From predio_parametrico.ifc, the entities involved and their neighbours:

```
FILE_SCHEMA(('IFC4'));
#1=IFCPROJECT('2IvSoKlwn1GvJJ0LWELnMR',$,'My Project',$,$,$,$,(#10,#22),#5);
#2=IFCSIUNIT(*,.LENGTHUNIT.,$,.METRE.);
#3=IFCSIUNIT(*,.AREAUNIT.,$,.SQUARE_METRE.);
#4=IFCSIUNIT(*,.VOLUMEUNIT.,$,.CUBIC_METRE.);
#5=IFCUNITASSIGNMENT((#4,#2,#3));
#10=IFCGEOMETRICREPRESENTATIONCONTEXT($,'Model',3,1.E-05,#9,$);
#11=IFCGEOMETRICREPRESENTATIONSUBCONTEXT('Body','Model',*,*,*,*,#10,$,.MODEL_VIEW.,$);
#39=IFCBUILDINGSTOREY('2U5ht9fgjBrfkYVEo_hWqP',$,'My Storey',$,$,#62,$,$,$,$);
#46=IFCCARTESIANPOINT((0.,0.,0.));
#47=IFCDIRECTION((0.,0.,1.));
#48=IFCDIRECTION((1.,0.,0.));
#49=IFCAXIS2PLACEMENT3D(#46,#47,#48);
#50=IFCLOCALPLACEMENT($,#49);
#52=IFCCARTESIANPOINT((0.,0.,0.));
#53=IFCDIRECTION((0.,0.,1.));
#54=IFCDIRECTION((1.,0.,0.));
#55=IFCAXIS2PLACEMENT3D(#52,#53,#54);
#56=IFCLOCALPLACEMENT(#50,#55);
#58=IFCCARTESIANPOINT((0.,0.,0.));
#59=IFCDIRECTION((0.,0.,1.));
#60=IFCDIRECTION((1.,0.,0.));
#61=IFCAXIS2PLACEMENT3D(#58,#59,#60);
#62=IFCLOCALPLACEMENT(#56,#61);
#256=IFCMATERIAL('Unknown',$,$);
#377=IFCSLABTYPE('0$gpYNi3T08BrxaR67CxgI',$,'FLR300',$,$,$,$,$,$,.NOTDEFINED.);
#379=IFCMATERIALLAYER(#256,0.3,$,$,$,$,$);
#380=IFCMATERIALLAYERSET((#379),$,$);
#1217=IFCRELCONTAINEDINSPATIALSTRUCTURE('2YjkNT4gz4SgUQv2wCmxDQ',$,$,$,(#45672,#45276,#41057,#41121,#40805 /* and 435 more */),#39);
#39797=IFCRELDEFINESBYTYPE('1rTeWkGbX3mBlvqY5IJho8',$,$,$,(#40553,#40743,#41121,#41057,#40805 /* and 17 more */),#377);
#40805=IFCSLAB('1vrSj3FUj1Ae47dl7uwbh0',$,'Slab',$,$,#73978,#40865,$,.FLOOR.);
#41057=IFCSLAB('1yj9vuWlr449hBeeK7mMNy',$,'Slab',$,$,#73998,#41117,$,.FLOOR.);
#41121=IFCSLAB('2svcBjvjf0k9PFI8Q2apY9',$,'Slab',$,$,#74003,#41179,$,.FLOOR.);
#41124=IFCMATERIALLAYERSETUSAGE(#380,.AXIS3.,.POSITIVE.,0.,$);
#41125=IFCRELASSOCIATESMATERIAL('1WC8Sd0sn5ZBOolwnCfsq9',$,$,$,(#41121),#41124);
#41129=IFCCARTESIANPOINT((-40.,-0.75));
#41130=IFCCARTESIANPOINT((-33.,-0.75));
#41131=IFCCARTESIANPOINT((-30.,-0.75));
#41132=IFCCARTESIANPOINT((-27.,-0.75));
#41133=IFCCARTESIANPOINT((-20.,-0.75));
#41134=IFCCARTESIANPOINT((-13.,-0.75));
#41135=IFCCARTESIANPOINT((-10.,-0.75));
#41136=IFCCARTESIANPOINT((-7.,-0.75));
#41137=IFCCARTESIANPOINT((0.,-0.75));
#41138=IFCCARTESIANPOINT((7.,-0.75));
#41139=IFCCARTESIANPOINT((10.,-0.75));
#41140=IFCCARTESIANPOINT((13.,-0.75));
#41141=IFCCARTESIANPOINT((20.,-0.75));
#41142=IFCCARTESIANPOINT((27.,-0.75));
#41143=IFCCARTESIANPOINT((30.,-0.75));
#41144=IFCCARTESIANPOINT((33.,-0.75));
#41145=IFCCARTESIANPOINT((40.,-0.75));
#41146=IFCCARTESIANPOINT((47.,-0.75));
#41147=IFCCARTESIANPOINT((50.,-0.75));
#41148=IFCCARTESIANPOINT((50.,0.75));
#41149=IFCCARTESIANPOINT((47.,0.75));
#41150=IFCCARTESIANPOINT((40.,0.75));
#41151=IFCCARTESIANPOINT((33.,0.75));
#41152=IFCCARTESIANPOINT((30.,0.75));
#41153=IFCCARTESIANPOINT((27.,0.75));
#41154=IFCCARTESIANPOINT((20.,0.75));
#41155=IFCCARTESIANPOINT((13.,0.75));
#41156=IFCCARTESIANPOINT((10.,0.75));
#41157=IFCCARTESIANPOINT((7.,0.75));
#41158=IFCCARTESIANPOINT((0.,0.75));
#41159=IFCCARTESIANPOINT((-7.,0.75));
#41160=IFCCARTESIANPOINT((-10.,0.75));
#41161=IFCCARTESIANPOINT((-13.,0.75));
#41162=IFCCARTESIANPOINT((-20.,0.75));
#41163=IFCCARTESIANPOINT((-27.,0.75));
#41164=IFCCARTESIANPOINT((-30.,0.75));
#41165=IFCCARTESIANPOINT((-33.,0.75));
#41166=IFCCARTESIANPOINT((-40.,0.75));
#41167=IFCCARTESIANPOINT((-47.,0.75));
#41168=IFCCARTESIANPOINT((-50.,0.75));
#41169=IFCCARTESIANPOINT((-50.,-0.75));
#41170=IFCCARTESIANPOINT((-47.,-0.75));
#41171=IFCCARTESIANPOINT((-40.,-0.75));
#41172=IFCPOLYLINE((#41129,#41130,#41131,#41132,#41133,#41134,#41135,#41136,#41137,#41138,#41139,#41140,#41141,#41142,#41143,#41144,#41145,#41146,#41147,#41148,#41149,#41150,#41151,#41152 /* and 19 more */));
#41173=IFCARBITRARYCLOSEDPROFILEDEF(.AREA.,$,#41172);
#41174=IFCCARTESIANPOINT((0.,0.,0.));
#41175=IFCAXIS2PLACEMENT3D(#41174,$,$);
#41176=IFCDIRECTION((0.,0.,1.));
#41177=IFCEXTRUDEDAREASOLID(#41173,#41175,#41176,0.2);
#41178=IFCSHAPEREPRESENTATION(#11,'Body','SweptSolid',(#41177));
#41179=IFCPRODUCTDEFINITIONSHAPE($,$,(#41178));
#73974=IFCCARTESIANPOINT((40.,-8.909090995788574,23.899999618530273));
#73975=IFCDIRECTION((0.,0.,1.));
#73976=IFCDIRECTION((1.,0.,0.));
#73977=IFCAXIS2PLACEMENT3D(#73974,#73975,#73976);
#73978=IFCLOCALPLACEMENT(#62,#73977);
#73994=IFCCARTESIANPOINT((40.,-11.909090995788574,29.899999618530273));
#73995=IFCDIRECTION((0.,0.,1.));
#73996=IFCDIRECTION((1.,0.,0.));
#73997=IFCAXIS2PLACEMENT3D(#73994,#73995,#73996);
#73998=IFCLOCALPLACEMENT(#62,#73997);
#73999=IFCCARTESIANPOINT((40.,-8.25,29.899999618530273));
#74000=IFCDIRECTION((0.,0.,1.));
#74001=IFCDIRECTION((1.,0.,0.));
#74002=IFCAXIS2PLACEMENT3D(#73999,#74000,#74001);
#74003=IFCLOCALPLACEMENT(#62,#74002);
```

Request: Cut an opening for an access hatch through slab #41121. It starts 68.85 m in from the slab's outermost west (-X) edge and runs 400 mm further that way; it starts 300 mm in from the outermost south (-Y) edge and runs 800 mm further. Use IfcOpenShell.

```python
import numpy as np
import ifcopenshell
import ifcopenshell.api.feature
import ifcopenshell.api.geometry
import ifcopenshell.api.root
import ifcopenshell.geom
import ifcopenshell.util.placement
import ifcopenshell.util.representation
import ifcopenshell.util.shape
import ifcopenshell.util.unit

model = ifcopenshell.open("predio_parametrico.ifc")
unit_scale = ifcopenshell.util.unit.calculate_unit_scale(model)
settings = ifcopenshell.geom.settings()


def volume(element):
    """Net volume in cubic metres, openings subtracted."""
    shape = ifcopenshell.geom.create_shape(settings, element)
    return ifcopenshell.util.shape.get_volume(shape.geometry)


slab = model.by_guid("2svcBjvjf0k9PFI8Q2apY9")
before = volume(slab)

# Extent in the slab's own axes, in metres. The edges named are its -X and -Y sides.
slab_shape = ifcopenshell.geom.create_shape(settings, slab)
vertices = ifcopenshell.util.shape.get_vertices(slab_shape.geometry)
x_min, y_min, bottom = vertices.min(axis=0)
top = vertices[:, 2].max()

opening = ifcopenshell.api.root.create_entity(model, ifc_class="IfcOpeningElement", name="Access hatch opening", predefined_type="OPENING")
context = ifcopenshell.util.representation.get_context(model, "Model", "Body", "MODEL_VIEW")
width, depth = 0.4, 0.8
outline = [(0.0, 0.0), (width, 0.0), (width, depth), (0.0, depth), (0.0, 0.0)]
# Overshoot both faces by 50 mm so the cut is clean.
shape = ifcopenshell.api.geometry.add_slab_representation(
    model, context=context, depth=top - bottom + 0.1, polyline=outline
)
ifcopenshell.api.geometry.assign_representation(model, product=opening, representation=shape)

matrix = ifcopenshell.util.placement.get_local_placement(slab.ObjectPlacement)
matrix[:, 3] = matrix @ np.append(np.array([x_min + 68.85, y_min + 0.3, bottom - 0.05]) / unit_scale, 1.0)
ifcopenshell.api.geometry.edit_object_placement(model, product=opening, matrix=matrix, is_si=False)
ifcopenshell.api.feature.add_feature(model, feature=opening, element=slab)

after = volume(slab)

print(f"slab volume {before:.3f} -> {after:.3f} m3")

model.write("predio_parametrico-out.ifc")
```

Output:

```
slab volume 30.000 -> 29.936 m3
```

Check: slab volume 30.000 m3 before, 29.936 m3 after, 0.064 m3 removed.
